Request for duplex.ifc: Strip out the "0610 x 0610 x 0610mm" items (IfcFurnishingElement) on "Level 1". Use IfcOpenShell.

First a look at what the model holds.

```python
import ifcopenshell
import ifcopenshell.util.element

model = ifcopenshell.open("duplex.ifc")
print(model.schema)
storey = next(s for s in model.by_type("IfcBuildingStorey") if s.Name == "Level 1")
furniture = [e for e in ifcopenshell.util.element.get_decomposition(storey) if e.is_a("IfcFurnishingElement")]
seen = {}
for e in furniture:
    element_type = ifcopenshell.util.element.get_type(e)
    name = element_type.Name if element_type not in (None, e) else None
    seen[name] = seen.get(name, 0) + 1
for name, count in sorted(seen.items(), key=str):
    print(count, "x", name)
```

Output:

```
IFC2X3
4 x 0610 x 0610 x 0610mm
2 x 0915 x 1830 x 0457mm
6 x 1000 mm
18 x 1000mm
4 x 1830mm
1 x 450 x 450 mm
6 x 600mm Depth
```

```python
import ifcopenshell
import ifcopenshell.api.root
import ifcopenshell.util.element

model = ifcopenshell.open("duplex.ifc")

storey = next(s for s in model.by_type("IfcBuildingStorey") if s.Name == "Level 1")
furniture = [e for e in ifcopenshell.util.element.get_decomposition(storey) if e.is_a("IfcFurnishingElement")]
targets = [e for e in furniture if (t := ifcopenshell.util.element.get_type(e)) not in (None, e) and t.Name == "0610 x 0610 x 0610mm"]

for e in targets:
    ifcopenshell.api.root.remove_product(model, product=e)
print(len(targets), "removed")

model.write("duplex-out.ifc")
```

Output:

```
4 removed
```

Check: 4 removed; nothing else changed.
